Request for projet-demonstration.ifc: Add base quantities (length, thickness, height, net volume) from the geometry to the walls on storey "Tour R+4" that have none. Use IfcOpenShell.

First a look at what the model holds.

```python
import ifcopenshell
import ifcopenshell.util.element
import ifcopenshell.util.unit

model = ifcopenshell.open("projet-demonstration.ifc")
print(model.schema)
for unit_type in ("LENGTHUNIT", "AREAUNIT", "VOLUMEUNIT"):
    print(unit_type, ifcopenshell.util.unit.calculate_unit_scale(model, unit_type))
storey = next(s for s in model.by_type("IfcBuildingStorey") if s.Name == "Tour R+4")
walls = [e for e in ifcopenshell.util.element.get_decomposition(storey) if e.is_a("IfcWall")]
for e in sorted(walls, key=lambda e: e.id()):
    print(e.id(), e.is_a(), e.Name, list(ifcopenshell.util.element.get_psets(e, qtos_only=True)), sep=" | ")
```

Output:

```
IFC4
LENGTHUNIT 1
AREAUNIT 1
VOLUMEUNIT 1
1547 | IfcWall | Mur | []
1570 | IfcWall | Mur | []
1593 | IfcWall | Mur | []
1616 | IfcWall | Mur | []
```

```python
import ifcopenshell
import ifcopenshell.api.pset
import ifcopenshell.geom
import ifcopenshell.util.element
import ifcopenshell.util.shape
import ifcopenshell.util.unit

model = ifcopenshell.open("projet-demonstration.ifc")
unit_scale = ifcopenshell.util.unit.calculate_unit_scale(model)
volume_scale = ifcopenshell.util.unit.calculate_unit_scale(model, "VOLUMEUNIT")
settings = ifcopenshell.geom.settings()

storey = next(s for s in model.by_type("IfcBuildingStorey") if s.Name == "Tour R+4")
walls = [e for e in ifcopenshell.util.element.get_decomposition(storey) if e.is_a("IfcWall")]

for e in sorted(walls, key=lambda e: e.id()):
    if ifcopenshell.util.element.get_psets(e, qtos_only=True, should_inherit=False):
        continue
    # Geometry comes back in metres, in the element's own axes.
    shape = ifcopenshell.geom.create_shape(settings, e)
    values = {
        "Length": ifcopenshell.util.shape.get_x(shape.geometry) / unit_scale,
        "Width": ifcopenshell.util.shape.get_y(shape.geometry) / unit_scale,
        "Height": ifcopenshell.util.shape.get_z(shape.geometry) / unit_scale,
        "NetVolume": ifcopenshell.util.shape.get_volume(shape.geometry) / volume_scale,
    }
    qto = ifcopenshell.api.pset.add_qto(model, product=e, name="Qto_WallBaseQuantities")
    ifcopenshell.api.pset.edit_qto(model, qto=qto, properties=values)
    print(e.id(), {k: round(v, 3) for k, v in values.items()})

model.write("projet-demonstration_rev.ifc")
```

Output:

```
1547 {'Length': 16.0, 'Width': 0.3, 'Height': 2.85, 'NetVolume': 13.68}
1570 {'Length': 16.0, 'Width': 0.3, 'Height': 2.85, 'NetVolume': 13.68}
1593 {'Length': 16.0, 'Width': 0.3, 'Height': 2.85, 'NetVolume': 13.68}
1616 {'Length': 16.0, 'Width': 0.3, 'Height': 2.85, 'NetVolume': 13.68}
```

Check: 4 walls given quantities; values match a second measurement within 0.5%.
